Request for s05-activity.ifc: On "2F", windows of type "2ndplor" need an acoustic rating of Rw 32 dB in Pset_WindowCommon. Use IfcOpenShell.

First a look at what the model holds.

```python
import ifcopenshell
import ifcopenshell.util.element

model = ifcopenshell.open("s05-activity.ifc")
print(model.schema)
storey = next(s for s in model.by_type("IfcBuildingStorey") if s.Name == "2F")
windows = [e for e in ifcopenshell.util.element.get_decomposition(storey) if e.is_a("IfcWindow")]
seen = {}
for e in windows:
    element_type = ifcopenshell.util.element.get_type(e)
    key = (element_type.Name if element_type != e and element_type else None, ifcopenshell.util.element.get_pset(e, "Pset_WindowCommon", "AcousticRating"))
    seen[key] = seen.get(key, 0) + 1
for (name, value), count in sorted(seen.items(), key=str):
    print(count, "x", name, "|", value)
```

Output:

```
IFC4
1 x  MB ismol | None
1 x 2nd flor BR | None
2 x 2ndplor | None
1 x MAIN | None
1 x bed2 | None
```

```python
import ifcopenshell
import ifcopenshell.api.pset
import ifcopenshell.util.element

model = ifcopenshell.open("s05-activity.ifc")

storey = next(s for s in model.by_type("IfcBuildingStorey") if s.Name == "2F")
windows = [e for e in ifcopenshell.util.element.get_decomposition(storey) if e.is_a("IfcWindow")]

count = 0
for e in windows:
    element_type = ifcopenshell.util.element.get_type(e)
    if element_type in (None, e) or element_type.Name != "2ndplor":
        continue
    # add_pset returns the element's existing set when there is one.
    pset = ifcopenshell.api.pset.add_pset(model, product=e, name="Pset_WindowCommon")
    ifcopenshell.api.pset.edit_pset(model, pset=pset, properties={"AcousticRating": "Rw 32 dB"})
    count += 1

print(count, "windows updated")

model.write("s05-activity_v2.ifc")
```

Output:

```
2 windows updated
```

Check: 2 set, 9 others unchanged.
